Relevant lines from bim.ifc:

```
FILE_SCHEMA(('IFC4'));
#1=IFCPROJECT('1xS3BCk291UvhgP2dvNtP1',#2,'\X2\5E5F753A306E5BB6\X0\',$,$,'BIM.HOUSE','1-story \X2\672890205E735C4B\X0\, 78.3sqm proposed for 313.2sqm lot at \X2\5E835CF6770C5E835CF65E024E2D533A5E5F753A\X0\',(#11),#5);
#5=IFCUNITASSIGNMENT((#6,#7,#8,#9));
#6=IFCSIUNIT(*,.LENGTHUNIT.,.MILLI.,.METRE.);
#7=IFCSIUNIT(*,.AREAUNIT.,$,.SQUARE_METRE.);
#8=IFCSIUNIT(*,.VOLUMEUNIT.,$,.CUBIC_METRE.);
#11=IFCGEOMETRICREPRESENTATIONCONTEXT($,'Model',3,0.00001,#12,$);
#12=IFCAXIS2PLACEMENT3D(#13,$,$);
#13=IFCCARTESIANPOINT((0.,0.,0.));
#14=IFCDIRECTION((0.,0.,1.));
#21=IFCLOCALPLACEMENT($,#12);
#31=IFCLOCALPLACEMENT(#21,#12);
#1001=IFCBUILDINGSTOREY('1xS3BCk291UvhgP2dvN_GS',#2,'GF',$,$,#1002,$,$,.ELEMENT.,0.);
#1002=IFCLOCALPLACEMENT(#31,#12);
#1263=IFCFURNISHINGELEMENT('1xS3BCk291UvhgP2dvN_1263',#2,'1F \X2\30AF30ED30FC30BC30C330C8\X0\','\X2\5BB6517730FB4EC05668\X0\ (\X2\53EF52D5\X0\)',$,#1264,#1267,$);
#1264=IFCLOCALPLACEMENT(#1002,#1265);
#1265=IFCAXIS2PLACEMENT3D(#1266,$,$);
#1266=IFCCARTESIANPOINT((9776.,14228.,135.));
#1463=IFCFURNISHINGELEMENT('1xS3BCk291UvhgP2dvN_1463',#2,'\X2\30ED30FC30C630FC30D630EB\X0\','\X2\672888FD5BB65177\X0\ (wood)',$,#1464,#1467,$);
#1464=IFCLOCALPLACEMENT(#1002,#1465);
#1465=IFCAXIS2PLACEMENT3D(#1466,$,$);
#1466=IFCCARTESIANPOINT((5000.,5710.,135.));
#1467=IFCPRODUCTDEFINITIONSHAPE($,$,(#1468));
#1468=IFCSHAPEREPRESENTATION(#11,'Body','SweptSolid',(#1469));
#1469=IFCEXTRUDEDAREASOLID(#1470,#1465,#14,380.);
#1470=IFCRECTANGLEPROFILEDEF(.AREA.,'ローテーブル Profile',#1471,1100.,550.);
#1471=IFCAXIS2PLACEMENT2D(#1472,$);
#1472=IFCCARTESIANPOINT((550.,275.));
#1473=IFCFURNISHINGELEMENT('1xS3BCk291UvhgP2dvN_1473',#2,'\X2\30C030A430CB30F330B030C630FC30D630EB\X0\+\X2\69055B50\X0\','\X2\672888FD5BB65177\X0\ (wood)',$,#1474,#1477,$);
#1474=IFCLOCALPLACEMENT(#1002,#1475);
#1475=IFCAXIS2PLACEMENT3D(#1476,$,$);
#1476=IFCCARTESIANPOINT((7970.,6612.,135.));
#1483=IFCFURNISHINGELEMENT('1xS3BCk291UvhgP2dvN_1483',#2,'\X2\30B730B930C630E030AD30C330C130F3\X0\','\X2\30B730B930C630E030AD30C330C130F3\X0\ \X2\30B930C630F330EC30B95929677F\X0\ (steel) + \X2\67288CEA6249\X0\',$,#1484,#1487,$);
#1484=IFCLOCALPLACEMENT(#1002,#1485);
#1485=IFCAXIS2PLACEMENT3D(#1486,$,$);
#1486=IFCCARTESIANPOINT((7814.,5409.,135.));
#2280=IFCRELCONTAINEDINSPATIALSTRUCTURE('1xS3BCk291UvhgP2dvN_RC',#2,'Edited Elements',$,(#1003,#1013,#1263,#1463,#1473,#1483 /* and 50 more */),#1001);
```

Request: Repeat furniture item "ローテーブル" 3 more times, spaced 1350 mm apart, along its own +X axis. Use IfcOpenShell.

```python
import ifcopenshell
import ifcopenshell.api.geometry
import ifcopenshell.api.root
import ifcopenshell.util.element
import ifcopenshell.util.placement
import ifcopenshell.util.unit

model = ifcopenshell.open("bim.ifc")
unit_scale = ifcopenshell.util.unit.calculate_unit_scale(model)


def reuse_history(source, copy):
    """copy_class also copies each property set's owner history, people and application; keep the originals."""
    for rel in copy.IsDefinedBy:
        if rel.is_a("IfcRelDefinesByProperties") and (history := rel.RelatingPropertyDefinition.OwnerHistory):
            rel.RelatingPropertyDefinition.OwnerHistory = source.OwnerHistory
            ifcopenshell.util.element.remove_deep2(model, history)


source = model.by_guid("1xS3BCk291UvhgP2dvN_1463")
base = ifcopenshell.util.placement.get_local_placement(source.ObjectPlacement)
step = base[:3, 0] * 1.35 / unit_scale

for i in range(1, 4):
    copy = ifcopenshell.api.root.copy_class(model, product=source)
    copy.Representation = ifcopenshell.util.element.copy_deep(
        model, source.Representation, exclude=["IfcGeometricRepresentationContext", "IfcRepresentationMap"]
    )
    reuse_history(source, copy)
    matrix = base.copy()
    matrix[:3, 3] += i * step
    print("added at", matrix[:3, 3].round(3) + 0.0)
    ifcopenshell.api.geometry.edit_object_placement(model, product=copy, matrix=matrix, is_si=False)

model.write("bim_edited.ifc")
```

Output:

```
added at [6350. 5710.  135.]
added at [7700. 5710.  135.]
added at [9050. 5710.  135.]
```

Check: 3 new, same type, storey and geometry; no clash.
